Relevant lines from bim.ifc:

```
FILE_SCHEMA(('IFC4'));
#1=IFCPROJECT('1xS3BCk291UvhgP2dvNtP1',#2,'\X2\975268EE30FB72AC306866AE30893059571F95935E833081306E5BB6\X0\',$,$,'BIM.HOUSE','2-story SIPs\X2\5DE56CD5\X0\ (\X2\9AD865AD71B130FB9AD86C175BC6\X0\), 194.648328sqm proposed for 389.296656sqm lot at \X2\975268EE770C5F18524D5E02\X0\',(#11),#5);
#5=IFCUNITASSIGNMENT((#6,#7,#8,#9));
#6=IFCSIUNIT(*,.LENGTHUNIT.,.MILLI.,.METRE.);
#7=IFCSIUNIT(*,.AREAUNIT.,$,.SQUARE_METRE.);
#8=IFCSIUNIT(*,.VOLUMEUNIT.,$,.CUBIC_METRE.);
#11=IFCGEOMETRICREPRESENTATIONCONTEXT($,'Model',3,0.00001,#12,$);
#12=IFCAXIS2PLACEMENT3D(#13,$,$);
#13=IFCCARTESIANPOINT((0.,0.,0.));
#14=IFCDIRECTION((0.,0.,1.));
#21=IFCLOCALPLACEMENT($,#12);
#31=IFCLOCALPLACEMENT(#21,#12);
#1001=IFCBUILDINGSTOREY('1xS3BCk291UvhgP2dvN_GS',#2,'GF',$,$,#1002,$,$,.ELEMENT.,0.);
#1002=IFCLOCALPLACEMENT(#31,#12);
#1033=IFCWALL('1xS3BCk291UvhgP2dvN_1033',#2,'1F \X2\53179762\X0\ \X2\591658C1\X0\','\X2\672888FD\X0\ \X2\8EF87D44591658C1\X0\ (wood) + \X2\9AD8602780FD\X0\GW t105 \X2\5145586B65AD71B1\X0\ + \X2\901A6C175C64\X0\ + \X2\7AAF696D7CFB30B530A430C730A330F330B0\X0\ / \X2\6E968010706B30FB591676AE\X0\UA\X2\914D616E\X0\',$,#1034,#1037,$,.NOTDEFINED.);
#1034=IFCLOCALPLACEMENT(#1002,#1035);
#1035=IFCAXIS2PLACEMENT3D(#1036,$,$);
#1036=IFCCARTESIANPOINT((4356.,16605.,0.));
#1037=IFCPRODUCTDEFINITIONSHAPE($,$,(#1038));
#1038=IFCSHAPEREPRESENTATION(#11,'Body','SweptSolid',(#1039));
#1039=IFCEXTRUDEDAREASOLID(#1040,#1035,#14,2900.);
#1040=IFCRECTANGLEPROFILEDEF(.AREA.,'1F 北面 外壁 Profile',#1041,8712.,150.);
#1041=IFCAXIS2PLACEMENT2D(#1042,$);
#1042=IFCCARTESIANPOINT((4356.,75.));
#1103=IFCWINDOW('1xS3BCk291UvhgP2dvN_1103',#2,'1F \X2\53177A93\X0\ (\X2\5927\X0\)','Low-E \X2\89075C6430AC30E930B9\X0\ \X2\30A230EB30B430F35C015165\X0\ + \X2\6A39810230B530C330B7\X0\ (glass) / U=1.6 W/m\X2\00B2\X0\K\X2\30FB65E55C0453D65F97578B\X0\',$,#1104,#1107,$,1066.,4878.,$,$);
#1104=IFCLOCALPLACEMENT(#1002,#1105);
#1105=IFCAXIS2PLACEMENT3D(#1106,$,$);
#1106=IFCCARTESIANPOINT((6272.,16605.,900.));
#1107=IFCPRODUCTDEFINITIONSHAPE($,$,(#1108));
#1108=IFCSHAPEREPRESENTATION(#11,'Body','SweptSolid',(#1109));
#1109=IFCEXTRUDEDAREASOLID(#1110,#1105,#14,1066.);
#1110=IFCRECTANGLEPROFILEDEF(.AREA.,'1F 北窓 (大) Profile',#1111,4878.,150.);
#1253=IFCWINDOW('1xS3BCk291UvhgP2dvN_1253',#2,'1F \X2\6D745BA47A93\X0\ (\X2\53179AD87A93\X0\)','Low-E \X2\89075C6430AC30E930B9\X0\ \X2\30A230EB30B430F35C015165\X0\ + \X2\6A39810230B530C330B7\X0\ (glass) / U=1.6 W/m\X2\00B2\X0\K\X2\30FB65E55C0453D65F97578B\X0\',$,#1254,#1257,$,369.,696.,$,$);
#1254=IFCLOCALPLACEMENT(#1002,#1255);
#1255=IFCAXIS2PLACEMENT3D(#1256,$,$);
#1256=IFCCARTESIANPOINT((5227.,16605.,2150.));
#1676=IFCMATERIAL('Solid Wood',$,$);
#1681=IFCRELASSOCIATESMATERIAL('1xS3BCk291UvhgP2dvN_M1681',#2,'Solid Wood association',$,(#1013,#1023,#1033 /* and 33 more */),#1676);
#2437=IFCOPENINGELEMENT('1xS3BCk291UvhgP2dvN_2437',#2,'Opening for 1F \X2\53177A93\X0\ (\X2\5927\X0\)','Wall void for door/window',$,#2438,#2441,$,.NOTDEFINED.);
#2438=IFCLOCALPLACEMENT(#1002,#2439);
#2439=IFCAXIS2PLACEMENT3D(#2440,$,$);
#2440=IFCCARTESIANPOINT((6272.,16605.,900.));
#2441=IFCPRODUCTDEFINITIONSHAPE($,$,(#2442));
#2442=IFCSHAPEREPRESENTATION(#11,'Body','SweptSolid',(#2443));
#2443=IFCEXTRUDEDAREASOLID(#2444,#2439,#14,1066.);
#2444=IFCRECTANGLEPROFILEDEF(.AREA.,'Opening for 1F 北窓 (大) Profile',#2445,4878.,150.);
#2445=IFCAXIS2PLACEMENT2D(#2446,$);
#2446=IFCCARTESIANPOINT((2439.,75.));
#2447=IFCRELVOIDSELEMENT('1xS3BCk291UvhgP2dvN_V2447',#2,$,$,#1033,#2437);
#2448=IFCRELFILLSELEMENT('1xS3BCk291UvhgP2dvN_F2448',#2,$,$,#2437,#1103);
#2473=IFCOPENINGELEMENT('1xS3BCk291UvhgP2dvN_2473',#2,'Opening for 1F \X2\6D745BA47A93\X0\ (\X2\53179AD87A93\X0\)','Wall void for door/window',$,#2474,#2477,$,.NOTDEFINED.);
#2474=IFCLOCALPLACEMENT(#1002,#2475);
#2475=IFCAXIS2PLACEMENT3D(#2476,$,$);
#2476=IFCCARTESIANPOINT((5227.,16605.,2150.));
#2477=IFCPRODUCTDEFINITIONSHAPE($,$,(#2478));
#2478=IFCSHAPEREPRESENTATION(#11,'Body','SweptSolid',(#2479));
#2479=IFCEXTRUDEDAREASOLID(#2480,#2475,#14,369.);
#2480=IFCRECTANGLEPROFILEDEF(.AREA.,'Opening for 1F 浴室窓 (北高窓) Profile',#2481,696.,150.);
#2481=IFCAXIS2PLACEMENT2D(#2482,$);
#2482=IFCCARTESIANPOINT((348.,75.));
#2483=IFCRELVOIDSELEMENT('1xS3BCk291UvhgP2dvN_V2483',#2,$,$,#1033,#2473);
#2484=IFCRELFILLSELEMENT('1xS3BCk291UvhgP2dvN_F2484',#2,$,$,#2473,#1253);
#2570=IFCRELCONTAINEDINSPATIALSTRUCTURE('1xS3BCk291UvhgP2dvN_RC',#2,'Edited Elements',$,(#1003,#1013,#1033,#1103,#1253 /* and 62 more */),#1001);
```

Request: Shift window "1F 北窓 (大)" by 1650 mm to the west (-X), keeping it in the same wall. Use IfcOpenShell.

```python
import ifcopenshell
import ifcopenshell.api.geometry
import ifcopenshell.util.placement
import ifcopenshell.util.unit

model = ifcopenshell.open("bim.ifc")
unit_scale = ifcopenshell.util.unit.calculate_unit_scale(model)

window = model.by_guid("1xS3BCk291UvhgP2dvN_1103")
opening = window.FillsVoids[0].RelatingOpeningElement
wall = opening.VoidsElements[0].RelatingBuildingElement

wall_matrix = ifcopenshell.util.placement.get_local_placement(wall.ObjectPlacement)
shift = wall_matrix[:3, 0] * -1.65 / unit_scale
before = ifcopenshell.util.placement.get_local_placement(window.ObjectPlacement)[:3, 3].copy()

# The window is not placed relative to its opening, so move both.
for product in (opening, window):
    matrix = ifcopenshell.util.placement.get_local_placement(product.ObjectPlacement)
    matrix[:3, 3] += shift
    ifcopenshell.api.geometry.edit_object_placement(model, product=product, matrix=matrix, is_si=False)

after = ifcopenshell.util.placement.get_local_placement(window.ObjectPlacement)[:3, 3]
print("window moved by", (after - before).round(3) + 0.0)

model.write("bim_rev.ifc")
```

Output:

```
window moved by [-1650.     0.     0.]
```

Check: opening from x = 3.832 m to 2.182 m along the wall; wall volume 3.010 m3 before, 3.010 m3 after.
